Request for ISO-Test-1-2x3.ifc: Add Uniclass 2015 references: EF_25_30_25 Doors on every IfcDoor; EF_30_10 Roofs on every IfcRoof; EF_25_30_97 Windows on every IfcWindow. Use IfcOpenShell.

First a look at what the model holds.

```python
import ifcopenshell

model = ifcopenshell.open("ISO-Test-1-2x3.ifc")
print(model.schema)
print("classifications:", [c.Name for c in model.by_type("IfcClassification")])
for ifc_class in ("IfcDoor", "IfcRoof", "IfcStair", "IfcWall", "IfcWindow"):
    print(ifc_class, len(model.by_type(ifc_class)))
```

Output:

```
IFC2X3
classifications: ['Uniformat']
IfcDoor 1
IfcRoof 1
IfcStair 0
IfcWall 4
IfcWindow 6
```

```python
import ifcopenshell
import ifcopenshell.api.classification

model = ifcopenshell.open("ISO-Test-1-2x3.ifc")

# IFC2X3 requires Source and Edition and has no link from the project to the system.
system = model.create_entity("IfcClassification", Source="NBS", Edition="2015", Name="Uniclass 2015")

codes = {
    "IfcDoor": ("EF_25_30_25", "Doors"),
    "IfcRoof": ("EF_30_10", "Roofs"),
    "IfcWindow": ("EF_25_30_97", "Windows"),
}
for ifc_class, (code, name) in codes.items():
    products = model.by_type(ifc_class)
    ifcopenshell.api.classification.add_reference(
        model, products=products, classification=system, identification=code, name=name
    )
    print(code, len(products))

model.write("ISO-Test-1-2x3-out.ifc")
```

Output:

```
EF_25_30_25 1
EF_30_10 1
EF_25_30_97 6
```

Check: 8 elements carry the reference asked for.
